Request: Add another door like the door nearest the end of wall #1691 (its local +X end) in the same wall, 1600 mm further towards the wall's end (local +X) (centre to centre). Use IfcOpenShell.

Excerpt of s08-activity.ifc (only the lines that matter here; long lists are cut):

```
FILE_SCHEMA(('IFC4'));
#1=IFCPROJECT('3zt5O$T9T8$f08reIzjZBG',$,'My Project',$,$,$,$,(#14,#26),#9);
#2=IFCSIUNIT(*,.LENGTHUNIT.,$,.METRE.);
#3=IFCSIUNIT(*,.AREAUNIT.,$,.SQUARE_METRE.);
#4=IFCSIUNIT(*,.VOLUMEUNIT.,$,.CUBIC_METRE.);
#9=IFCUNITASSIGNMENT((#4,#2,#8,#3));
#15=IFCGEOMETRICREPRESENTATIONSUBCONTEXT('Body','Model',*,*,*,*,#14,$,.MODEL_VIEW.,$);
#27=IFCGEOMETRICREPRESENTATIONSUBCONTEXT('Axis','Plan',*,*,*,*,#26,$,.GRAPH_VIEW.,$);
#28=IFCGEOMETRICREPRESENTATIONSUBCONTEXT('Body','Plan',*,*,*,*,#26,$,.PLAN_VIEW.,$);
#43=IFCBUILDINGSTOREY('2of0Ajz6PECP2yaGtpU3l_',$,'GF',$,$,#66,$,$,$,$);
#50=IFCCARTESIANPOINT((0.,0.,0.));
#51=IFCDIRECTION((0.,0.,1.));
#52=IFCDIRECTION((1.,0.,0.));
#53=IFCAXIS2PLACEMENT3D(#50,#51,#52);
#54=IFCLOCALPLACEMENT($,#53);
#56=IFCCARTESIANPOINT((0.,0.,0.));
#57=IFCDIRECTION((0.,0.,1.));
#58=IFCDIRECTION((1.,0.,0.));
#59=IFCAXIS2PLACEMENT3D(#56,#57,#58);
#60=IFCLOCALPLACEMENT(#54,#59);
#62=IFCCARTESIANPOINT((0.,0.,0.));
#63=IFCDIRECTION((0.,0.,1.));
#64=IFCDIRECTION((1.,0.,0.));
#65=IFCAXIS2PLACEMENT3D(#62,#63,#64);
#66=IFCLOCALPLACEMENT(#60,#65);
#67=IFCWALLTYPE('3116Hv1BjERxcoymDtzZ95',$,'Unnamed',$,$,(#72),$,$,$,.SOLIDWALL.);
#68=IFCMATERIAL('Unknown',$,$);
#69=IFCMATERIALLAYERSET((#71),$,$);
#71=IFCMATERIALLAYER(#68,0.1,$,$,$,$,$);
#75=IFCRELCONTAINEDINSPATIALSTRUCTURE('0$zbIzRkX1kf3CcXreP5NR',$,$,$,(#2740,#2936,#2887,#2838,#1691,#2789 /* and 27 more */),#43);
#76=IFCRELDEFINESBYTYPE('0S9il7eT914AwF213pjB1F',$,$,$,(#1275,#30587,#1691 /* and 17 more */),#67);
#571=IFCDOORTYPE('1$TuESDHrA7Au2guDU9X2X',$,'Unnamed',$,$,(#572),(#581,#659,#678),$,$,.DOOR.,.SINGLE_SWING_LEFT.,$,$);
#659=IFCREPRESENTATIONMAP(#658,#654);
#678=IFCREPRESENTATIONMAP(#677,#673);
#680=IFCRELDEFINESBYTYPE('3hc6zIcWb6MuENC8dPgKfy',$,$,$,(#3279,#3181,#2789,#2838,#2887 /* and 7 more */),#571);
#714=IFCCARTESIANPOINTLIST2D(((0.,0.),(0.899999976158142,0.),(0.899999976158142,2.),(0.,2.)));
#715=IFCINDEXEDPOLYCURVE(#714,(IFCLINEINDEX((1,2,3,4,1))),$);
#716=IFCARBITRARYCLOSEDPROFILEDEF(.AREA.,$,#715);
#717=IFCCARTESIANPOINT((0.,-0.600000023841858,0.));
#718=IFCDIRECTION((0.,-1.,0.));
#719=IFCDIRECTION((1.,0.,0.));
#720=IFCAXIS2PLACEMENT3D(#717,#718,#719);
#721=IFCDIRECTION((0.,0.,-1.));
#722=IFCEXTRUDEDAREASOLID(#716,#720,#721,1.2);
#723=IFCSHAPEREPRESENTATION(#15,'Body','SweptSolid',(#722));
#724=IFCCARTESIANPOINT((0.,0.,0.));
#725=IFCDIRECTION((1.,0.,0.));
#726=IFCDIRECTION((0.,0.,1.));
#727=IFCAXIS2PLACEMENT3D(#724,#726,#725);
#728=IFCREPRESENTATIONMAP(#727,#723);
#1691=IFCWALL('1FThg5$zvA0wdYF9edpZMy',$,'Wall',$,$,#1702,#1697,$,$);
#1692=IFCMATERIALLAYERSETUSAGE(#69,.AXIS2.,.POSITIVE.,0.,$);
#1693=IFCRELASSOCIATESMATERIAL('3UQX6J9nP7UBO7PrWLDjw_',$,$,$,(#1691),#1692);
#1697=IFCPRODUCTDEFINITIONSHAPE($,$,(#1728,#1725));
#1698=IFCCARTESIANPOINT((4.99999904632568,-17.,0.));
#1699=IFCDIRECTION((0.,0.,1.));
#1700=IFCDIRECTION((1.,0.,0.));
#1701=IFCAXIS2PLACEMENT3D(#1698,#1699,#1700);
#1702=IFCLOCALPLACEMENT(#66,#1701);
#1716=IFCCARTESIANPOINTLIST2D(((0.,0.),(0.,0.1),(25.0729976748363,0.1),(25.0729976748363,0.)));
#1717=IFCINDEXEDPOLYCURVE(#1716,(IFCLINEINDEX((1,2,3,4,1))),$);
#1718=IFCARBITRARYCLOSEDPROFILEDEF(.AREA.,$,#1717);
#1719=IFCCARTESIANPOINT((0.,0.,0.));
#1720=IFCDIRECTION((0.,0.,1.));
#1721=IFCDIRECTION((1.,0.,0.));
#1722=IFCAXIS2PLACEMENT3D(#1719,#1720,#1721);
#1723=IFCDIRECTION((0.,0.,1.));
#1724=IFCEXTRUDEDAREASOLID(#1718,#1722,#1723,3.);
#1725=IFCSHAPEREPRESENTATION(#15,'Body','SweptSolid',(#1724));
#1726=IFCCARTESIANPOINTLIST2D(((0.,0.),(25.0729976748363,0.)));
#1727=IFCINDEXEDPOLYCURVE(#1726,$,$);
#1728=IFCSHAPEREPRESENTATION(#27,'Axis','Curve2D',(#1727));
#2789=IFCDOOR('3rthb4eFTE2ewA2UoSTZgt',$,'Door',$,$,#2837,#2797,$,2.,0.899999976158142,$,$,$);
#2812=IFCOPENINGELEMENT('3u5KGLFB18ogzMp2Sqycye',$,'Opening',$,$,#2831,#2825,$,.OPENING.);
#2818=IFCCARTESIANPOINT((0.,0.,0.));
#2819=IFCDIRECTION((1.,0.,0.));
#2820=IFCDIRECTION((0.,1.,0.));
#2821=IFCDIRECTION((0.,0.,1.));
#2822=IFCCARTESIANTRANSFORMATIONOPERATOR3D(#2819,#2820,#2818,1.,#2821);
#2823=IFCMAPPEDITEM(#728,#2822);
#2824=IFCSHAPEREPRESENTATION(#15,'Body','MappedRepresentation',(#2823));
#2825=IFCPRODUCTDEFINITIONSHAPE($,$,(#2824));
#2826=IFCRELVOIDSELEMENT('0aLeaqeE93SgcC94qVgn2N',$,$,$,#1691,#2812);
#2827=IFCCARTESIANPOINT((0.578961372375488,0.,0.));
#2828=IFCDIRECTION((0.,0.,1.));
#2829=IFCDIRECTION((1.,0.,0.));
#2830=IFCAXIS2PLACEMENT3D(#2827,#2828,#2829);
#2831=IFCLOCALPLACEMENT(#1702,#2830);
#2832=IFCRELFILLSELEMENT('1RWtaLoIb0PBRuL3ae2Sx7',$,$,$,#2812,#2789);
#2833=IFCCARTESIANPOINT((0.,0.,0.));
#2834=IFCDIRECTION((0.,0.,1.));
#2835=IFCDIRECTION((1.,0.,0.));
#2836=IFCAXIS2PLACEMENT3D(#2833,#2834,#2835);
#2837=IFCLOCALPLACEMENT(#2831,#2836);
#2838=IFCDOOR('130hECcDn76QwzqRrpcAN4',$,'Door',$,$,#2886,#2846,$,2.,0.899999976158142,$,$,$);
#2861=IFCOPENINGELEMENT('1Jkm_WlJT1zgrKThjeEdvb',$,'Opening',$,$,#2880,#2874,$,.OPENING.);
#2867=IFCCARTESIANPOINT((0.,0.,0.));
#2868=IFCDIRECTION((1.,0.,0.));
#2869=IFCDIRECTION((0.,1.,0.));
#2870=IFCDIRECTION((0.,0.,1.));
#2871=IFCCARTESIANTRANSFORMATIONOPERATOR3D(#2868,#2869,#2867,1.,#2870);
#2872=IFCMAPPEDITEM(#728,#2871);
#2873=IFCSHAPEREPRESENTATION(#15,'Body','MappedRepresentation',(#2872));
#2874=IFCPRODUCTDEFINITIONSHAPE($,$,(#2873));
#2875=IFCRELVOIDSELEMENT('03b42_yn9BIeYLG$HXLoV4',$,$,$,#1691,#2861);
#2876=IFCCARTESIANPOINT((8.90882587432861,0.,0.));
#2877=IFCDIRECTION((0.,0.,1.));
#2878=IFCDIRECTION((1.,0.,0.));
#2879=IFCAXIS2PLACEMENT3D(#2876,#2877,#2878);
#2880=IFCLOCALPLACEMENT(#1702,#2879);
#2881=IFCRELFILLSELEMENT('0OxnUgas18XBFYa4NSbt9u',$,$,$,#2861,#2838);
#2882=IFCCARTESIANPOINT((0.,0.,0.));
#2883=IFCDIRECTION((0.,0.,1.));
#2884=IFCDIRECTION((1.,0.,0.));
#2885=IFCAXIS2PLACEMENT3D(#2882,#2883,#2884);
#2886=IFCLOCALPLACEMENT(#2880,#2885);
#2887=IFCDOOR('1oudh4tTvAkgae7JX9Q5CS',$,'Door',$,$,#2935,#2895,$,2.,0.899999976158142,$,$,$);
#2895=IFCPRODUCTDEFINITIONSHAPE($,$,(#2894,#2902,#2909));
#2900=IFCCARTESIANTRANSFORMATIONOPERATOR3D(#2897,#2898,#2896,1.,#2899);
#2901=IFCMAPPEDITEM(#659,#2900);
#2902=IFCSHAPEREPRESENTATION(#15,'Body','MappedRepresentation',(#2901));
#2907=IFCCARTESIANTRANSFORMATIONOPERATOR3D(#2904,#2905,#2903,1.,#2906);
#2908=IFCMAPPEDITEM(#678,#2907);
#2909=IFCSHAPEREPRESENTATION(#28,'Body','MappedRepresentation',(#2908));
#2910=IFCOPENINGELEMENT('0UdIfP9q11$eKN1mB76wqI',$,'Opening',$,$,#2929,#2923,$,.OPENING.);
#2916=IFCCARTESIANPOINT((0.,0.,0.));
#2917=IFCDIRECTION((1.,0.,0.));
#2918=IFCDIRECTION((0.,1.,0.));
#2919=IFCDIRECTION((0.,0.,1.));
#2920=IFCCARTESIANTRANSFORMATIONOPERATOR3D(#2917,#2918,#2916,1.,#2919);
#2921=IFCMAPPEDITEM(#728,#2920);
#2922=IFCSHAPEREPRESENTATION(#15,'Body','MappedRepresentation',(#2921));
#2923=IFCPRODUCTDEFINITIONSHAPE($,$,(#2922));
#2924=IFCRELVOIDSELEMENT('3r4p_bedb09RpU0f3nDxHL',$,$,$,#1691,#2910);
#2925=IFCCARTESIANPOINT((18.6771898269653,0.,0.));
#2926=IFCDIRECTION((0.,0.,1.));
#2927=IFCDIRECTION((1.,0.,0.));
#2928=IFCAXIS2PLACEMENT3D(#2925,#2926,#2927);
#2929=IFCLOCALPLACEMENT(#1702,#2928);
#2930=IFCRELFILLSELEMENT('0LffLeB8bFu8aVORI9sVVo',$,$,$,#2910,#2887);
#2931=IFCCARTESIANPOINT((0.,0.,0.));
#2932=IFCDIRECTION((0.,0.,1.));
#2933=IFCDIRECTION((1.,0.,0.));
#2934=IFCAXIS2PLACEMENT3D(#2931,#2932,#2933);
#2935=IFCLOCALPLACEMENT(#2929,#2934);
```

```python
import ifcopenshell
import ifcopenshell.api.feature
import ifcopenshell.api.geometry
import ifcopenshell.api.root
import ifcopenshell.geom
import ifcopenshell.util.element
import ifcopenshell.util.placement
import ifcopenshell.util.shape

model = ifcopenshell.open("s08-activity.ifc")
settings = ifcopenshell.geom.settings()


def volume(element):
    """Net volume in cubic metres, openings subtracted."""
    shape = ifcopenshell.geom.create_shape(settings, element)
    return ifcopenshell.util.shape.get_volume(shape.geometry)


door = model.by_guid("1oudh4tTvAkgae7JX9Q5CS")
opening = door.FillsVoids[0].RelatingOpeningElement
wall = opening.VoidsElements[0].RelatingBuildingElement
before = volume(wall)
shift = ifcopenshell.util.placement.get_local_placement(wall.ObjectPlacement)[:3, 0] * 1.6

# copy_class copies the void relationship, type, container and properties, but no geometry.
new_opening = ifcopenshell.api.root.copy_class(model, product=opening)
new_opening.Representation = ifcopenshell.util.element.copy_deep(
    model, opening.Representation, exclude=["IfcGeometricRepresentationContext", "IfcRepresentationMap"]
)
new_door = ifcopenshell.api.root.copy_class(model, product=door)
new_door.Representation = ifcopenshell.util.element.copy_deep(
    model, door.Representation, exclude=["IfcGeometricRepresentationContext", "IfcRepresentationMap"]
)
ifcopenshell.api.feature.add_filling(model, opening=new_opening, element=new_door)

for old, new in ((opening, new_opening), (door, new_door)):
    matrix = ifcopenshell.util.placement.get_local_placement(old.ObjectPlacement)
    matrix[:3, 3] += shift
    ifcopenshell.api.geometry.edit_object_placement(model, product=new, matrix=matrix, is_si=False)

after = volume(wall)

print(f"wall volume {before:.3f} -> {after:.3f} m3")

model.write("s08-activity_rev.ifc")
```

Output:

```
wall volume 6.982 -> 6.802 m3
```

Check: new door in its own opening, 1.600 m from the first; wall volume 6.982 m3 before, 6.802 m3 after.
